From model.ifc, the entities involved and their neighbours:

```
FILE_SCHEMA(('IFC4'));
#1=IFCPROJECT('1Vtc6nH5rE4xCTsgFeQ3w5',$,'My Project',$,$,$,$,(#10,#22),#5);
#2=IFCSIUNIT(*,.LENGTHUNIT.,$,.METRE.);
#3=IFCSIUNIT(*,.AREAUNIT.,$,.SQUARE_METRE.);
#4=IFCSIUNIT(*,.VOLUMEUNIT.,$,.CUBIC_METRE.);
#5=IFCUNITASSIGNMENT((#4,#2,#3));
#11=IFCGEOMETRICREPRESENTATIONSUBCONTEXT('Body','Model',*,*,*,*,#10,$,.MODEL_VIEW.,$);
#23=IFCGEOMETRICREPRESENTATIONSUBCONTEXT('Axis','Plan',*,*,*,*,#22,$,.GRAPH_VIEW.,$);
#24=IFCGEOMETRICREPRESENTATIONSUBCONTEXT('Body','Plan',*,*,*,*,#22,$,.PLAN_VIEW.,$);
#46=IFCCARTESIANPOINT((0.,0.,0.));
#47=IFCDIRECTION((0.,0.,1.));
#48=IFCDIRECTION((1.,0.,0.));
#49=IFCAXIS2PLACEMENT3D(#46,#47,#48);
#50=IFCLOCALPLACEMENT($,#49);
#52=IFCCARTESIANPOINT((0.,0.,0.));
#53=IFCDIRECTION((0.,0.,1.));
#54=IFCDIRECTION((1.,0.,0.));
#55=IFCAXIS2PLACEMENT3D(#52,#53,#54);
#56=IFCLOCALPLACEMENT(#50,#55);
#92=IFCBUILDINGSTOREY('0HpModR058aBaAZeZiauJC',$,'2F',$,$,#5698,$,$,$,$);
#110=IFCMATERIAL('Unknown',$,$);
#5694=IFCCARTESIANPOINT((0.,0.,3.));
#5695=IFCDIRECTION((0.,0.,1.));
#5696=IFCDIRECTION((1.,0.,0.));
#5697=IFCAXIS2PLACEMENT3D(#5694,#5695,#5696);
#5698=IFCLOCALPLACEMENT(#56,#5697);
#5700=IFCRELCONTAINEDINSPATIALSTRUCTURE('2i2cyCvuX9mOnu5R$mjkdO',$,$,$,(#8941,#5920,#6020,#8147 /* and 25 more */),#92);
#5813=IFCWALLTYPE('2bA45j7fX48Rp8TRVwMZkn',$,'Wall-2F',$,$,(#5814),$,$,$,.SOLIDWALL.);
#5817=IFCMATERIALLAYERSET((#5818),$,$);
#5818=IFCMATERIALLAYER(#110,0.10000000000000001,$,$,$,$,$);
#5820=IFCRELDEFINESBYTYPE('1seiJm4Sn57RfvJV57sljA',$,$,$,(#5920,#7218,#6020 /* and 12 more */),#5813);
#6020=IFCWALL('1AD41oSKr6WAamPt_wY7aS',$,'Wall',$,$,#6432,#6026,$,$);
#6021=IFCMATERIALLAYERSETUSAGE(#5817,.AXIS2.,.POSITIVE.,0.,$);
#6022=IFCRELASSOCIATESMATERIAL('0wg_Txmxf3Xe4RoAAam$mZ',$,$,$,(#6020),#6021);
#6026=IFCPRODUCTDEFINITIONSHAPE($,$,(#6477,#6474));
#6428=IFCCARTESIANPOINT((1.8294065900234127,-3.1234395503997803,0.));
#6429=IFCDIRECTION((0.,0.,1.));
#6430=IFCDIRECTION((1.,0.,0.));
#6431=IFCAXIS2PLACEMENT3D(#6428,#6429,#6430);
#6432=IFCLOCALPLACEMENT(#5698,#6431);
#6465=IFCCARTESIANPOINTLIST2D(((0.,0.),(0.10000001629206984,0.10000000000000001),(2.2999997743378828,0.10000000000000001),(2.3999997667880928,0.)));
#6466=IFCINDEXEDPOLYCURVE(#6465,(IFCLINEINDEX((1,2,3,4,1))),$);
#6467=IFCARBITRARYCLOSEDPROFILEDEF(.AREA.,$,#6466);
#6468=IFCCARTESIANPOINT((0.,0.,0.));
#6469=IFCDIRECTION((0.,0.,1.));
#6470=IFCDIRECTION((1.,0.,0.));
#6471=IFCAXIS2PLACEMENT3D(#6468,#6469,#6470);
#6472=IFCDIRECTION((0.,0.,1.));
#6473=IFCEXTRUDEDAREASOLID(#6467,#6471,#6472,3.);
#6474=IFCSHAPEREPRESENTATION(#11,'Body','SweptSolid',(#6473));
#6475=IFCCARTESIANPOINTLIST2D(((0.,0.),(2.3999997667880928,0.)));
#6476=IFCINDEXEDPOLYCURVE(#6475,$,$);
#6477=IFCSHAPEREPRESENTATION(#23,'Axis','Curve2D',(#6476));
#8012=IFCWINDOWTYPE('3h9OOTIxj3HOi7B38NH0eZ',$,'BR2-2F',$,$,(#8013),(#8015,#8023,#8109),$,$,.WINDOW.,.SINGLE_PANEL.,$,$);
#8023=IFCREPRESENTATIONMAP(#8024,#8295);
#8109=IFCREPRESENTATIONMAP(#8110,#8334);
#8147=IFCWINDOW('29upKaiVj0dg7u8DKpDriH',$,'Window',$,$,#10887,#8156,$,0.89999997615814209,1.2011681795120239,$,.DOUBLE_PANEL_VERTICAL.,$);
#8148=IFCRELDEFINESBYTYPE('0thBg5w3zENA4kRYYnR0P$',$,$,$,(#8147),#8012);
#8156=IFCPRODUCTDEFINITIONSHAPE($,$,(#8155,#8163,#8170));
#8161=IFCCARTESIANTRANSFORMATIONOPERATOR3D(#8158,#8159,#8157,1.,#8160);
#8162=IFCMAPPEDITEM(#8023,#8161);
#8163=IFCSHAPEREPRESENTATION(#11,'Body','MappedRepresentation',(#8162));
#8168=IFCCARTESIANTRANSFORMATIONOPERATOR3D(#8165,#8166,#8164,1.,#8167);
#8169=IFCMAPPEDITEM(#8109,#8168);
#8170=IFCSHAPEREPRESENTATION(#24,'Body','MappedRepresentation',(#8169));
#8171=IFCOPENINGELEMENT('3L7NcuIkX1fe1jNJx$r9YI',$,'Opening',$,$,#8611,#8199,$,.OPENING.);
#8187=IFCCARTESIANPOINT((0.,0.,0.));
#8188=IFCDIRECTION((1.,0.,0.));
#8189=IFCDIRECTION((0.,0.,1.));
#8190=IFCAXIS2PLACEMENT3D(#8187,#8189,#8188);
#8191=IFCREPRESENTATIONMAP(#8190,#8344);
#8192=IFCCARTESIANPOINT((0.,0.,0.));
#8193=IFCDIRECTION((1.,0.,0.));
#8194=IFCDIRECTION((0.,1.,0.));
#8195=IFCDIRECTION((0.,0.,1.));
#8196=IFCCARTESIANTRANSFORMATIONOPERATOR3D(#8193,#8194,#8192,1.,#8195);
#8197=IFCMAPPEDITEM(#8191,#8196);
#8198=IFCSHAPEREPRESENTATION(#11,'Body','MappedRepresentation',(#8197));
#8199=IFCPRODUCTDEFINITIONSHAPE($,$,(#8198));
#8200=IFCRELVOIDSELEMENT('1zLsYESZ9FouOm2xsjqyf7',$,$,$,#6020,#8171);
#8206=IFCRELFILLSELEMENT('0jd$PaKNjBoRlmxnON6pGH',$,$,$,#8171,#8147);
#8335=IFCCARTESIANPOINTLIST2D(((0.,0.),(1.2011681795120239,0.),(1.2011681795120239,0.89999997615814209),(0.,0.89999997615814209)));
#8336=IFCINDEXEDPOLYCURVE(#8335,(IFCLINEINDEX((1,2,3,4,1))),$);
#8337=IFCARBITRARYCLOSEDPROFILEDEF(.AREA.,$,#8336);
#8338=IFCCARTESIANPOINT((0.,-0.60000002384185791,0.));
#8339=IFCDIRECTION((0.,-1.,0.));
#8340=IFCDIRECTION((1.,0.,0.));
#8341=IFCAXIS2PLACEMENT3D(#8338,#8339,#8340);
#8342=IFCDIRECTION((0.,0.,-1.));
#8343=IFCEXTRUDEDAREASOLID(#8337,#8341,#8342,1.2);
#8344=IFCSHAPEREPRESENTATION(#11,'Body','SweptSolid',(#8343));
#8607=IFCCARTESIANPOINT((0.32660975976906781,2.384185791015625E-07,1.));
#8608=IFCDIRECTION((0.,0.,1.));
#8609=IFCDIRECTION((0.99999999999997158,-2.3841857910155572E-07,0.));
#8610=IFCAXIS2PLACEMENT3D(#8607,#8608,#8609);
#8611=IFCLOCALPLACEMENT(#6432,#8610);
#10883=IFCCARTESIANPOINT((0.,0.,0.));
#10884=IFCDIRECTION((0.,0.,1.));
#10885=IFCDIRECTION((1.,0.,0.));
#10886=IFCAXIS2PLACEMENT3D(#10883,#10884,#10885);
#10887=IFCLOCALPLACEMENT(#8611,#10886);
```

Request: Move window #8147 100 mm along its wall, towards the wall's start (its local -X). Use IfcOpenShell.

```python
import ifcopenshell
import ifcopenshell.api.geometry
import ifcopenshell.util.placement
import ifcopenshell.util.unit

model = ifcopenshell.open("model.ifc")
unit_scale = ifcopenshell.util.unit.calculate_unit_scale(model)

window = model.by_id(8147)
opening = window.FillsVoids[0].RelatingOpeningElement
wall = opening.VoidsElements[0].RelatingBuildingElement

wall_matrix = ifcopenshell.util.placement.get_local_placement(wall.ObjectPlacement)
shift = wall_matrix[:3, 0] * -0.1 / unit_scale
before = ifcopenshell.util.placement.get_local_placement(window.ObjectPlacement)[:3, 3].copy()

# The window is placed relative to its opening, so it follows when the opening moves.
matrix = ifcopenshell.util.placement.get_local_placement(opening.ObjectPlacement)
matrix[:3, 3] += shift
ifcopenshell.api.geometry.edit_object_placement(
    model, product=opening, matrix=matrix, is_si=False, should_transform_children=True
)

after = ifcopenshell.util.placement.get_local_placement(window.ObjectPlacement)[:3, 3]
print("window moved by", (after - before).round(3) + 0.0)

model.write("model-out.ifc")
```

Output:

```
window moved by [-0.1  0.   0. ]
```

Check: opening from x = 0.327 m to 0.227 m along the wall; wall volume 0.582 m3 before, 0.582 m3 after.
